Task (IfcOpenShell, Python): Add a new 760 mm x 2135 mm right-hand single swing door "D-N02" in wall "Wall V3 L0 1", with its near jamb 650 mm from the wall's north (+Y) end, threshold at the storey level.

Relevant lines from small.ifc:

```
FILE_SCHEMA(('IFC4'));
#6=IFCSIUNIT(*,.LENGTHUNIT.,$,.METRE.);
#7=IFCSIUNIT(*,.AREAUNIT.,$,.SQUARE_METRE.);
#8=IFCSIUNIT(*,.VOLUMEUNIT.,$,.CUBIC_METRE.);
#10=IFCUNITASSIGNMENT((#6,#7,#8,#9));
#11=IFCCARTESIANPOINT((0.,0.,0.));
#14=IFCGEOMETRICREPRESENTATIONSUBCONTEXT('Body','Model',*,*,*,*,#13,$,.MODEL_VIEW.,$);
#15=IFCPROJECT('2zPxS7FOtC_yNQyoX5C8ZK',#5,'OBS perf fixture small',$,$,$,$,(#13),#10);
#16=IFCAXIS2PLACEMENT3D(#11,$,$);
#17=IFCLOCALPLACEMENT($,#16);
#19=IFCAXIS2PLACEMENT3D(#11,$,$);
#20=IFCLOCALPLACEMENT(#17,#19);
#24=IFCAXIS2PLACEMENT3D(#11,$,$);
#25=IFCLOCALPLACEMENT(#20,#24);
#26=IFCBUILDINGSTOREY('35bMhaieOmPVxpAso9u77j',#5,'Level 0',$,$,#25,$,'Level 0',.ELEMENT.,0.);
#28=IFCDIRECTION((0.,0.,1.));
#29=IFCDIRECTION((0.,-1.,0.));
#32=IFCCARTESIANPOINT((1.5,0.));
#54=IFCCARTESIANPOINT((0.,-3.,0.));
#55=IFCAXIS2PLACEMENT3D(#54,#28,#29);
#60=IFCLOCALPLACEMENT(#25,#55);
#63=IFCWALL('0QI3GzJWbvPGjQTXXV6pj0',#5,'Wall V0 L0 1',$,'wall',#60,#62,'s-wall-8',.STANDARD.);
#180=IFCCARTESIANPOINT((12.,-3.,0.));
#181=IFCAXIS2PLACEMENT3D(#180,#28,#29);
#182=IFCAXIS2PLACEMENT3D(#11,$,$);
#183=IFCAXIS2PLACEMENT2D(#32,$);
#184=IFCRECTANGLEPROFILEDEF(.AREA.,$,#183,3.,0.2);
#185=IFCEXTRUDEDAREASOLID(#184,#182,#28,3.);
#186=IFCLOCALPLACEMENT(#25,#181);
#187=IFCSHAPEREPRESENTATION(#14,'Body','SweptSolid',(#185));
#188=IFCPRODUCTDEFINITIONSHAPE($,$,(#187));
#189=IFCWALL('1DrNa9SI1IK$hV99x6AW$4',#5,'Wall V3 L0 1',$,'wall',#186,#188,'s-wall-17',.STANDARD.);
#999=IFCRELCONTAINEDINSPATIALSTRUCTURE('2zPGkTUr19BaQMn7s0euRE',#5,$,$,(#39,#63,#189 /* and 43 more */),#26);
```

```python
import numpy as np
import ifcopenshell
import ifcopenshell.api.feature
import ifcopenshell.api.geometry
import ifcopenshell.api.root
import ifcopenshell.api.spatial
import ifcopenshell.geom
import ifcopenshell.util.element
import ifcopenshell.util.placement
import ifcopenshell.util.representation
import ifcopenshell.util.shape
import ifcopenshell.util.unit

model = ifcopenshell.open("small.ifc")
unit_scale = ifcopenshell.util.unit.calculate_unit_scale(model)
settings = ifcopenshell.geom.settings()


def volume(element):
    """Net volume in cubic metres, openings subtracted."""
    shape = ifcopenshell.geom.create_shape(settings, element)
    return ifcopenshell.util.shape.get_volume(shape.geometry)


wall = model.by_guid("1DrNa9SI1IK$hV99x6AW$4")
storey = ifcopenshell.util.element.get_container(wall, ifc_class="IfcBuildingStorey")
context = ifcopenshell.util.representation.get_context(model, "Model", "Body", "MODEL_VIEW")
before = volume(wall)

width, height, from_end, sill = 0.76, 2.135, 0.65, 0.0  # metres

# The wall runs along its own X axis, and the end named is its -X end.
wall_shape = ifcopenshell.geom.create_shape(settings, wall)
x, y, z = ifcopenshell.util.shape.get_vertices(wall_shape.geometry).T
start = x.min() + from_end
face, thickness = float(y.min()), float(y.max() - y.min())
wall_matrix = ifcopenshell.util.placement.get_local_placement(wall.ObjectPlacement)
level = ifcopenshell.util.placement.get_local_placement(storey.ObjectPlacement)[2, 3]


def in_wall(x, y):
    """Placement at x, y metres in the wall's axes, at sill height."""
    matrix = wall_matrix.copy()
    matrix[:, 3] = wall_matrix @ np.array([x / unit_scale, y / unit_scale, 0.0, 1.0])
    matrix[2, 3] = level + sill / unit_scale
    return matrix


# Opening: a box that overshoots both wall faces by 50 mm.
opening = ifcopenshell.api.root.create_entity(model, ifc_class="IfcOpeningElement", predefined_type="OPENING")
box = ifcopenshell.api.geometry.add_wall_representation(
    model, context=context, length=width, height=height, thickness=thickness + 0.1
)
ifcopenshell.api.geometry.assign_representation(model, product=opening, representation=box)
ifcopenshell.api.geometry.edit_object_placement(model, product=opening, matrix=in_wall(start, face - 0.05), is_si=False)
ifcopenshell.api.feature.add_feature(model, feature=opening, element=wall)

door = ifcopenshell.api.root.create_entity(model, ifc_class="IfcDoor", name="D-N02", predefined_type="DOOR")
door.OverallWidth, door.OverallHeight = width / unit_scale, height / unit_scale
door.OperationType = "SINGLE_SWING_RIGHT"
body = ifcopenshell.api.geometry.add_door_representation(
    model,
    context=context,
    overall_width=door.OverallWidth,
    overall_height=door.OverallHeight,
    operation_type="SINGLE_SWING_RIGHT",
    lining_properties={"LiningDepth": thickness / unit_scale, "ThresholdDepth": thickness / unit_scale},
)
ifcopenshell.api.geometry.assign_representation(model, product=door, representation=body)
ifcopenshell.api.spatial.assign_container(model, products=[door], relating_structure=storey)
ifcopenshell.api.feature.add_filling(model, opening=opening, element=door)

# The lining spans the wall, so the door starts at the wall face.
ifcopenshell.api.geometry.edit_object_placement(model, product=door, matrix=in_wall(start, face), is_si=False)

after = volume(wall)

print(f"wall volume {before:.3f} -> {after:.3f} m3")

model.write("small_rev.ifc")
```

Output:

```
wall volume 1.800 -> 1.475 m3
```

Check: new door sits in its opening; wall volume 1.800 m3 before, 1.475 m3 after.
